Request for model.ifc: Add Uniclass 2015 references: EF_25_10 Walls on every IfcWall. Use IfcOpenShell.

First a look at what the model holds.

```python
import ifcopenshell

model = ifcopenshell.open("model.ifc")
print(model.schema)
print("classifications:", [c.Name for c in model.by_type("IfcClassification")])
for ifc_class in ("IfcDoor", "IfcRoof", "IfcStair", "IfcWall", "IfcWindow"):
    print(ifc_class, len(model.by_type(ifc_class)))
```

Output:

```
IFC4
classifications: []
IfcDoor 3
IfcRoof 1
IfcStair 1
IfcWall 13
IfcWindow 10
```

```python
import ifcopenshell
import ifcopenshell.api.classification

model = ifcopenshell.open("model.ifc")

system = ifcopenshell.api.classification.add_classification(model, classification="Uniclass 2015")

codes = {
    "IfcWall": ("EF_25_10", "Walls"),
}
for ifc_class, (code, name) in codes.items():
    products = model.by_type(ifc_class)
    ifcopenshell.api.classification.add_reference(
        model, products=products, classification=system, identification=code, name=name
    )
    print(code, len(products))

model.write("model_updated.ifc")
```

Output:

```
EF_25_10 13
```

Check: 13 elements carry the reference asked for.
